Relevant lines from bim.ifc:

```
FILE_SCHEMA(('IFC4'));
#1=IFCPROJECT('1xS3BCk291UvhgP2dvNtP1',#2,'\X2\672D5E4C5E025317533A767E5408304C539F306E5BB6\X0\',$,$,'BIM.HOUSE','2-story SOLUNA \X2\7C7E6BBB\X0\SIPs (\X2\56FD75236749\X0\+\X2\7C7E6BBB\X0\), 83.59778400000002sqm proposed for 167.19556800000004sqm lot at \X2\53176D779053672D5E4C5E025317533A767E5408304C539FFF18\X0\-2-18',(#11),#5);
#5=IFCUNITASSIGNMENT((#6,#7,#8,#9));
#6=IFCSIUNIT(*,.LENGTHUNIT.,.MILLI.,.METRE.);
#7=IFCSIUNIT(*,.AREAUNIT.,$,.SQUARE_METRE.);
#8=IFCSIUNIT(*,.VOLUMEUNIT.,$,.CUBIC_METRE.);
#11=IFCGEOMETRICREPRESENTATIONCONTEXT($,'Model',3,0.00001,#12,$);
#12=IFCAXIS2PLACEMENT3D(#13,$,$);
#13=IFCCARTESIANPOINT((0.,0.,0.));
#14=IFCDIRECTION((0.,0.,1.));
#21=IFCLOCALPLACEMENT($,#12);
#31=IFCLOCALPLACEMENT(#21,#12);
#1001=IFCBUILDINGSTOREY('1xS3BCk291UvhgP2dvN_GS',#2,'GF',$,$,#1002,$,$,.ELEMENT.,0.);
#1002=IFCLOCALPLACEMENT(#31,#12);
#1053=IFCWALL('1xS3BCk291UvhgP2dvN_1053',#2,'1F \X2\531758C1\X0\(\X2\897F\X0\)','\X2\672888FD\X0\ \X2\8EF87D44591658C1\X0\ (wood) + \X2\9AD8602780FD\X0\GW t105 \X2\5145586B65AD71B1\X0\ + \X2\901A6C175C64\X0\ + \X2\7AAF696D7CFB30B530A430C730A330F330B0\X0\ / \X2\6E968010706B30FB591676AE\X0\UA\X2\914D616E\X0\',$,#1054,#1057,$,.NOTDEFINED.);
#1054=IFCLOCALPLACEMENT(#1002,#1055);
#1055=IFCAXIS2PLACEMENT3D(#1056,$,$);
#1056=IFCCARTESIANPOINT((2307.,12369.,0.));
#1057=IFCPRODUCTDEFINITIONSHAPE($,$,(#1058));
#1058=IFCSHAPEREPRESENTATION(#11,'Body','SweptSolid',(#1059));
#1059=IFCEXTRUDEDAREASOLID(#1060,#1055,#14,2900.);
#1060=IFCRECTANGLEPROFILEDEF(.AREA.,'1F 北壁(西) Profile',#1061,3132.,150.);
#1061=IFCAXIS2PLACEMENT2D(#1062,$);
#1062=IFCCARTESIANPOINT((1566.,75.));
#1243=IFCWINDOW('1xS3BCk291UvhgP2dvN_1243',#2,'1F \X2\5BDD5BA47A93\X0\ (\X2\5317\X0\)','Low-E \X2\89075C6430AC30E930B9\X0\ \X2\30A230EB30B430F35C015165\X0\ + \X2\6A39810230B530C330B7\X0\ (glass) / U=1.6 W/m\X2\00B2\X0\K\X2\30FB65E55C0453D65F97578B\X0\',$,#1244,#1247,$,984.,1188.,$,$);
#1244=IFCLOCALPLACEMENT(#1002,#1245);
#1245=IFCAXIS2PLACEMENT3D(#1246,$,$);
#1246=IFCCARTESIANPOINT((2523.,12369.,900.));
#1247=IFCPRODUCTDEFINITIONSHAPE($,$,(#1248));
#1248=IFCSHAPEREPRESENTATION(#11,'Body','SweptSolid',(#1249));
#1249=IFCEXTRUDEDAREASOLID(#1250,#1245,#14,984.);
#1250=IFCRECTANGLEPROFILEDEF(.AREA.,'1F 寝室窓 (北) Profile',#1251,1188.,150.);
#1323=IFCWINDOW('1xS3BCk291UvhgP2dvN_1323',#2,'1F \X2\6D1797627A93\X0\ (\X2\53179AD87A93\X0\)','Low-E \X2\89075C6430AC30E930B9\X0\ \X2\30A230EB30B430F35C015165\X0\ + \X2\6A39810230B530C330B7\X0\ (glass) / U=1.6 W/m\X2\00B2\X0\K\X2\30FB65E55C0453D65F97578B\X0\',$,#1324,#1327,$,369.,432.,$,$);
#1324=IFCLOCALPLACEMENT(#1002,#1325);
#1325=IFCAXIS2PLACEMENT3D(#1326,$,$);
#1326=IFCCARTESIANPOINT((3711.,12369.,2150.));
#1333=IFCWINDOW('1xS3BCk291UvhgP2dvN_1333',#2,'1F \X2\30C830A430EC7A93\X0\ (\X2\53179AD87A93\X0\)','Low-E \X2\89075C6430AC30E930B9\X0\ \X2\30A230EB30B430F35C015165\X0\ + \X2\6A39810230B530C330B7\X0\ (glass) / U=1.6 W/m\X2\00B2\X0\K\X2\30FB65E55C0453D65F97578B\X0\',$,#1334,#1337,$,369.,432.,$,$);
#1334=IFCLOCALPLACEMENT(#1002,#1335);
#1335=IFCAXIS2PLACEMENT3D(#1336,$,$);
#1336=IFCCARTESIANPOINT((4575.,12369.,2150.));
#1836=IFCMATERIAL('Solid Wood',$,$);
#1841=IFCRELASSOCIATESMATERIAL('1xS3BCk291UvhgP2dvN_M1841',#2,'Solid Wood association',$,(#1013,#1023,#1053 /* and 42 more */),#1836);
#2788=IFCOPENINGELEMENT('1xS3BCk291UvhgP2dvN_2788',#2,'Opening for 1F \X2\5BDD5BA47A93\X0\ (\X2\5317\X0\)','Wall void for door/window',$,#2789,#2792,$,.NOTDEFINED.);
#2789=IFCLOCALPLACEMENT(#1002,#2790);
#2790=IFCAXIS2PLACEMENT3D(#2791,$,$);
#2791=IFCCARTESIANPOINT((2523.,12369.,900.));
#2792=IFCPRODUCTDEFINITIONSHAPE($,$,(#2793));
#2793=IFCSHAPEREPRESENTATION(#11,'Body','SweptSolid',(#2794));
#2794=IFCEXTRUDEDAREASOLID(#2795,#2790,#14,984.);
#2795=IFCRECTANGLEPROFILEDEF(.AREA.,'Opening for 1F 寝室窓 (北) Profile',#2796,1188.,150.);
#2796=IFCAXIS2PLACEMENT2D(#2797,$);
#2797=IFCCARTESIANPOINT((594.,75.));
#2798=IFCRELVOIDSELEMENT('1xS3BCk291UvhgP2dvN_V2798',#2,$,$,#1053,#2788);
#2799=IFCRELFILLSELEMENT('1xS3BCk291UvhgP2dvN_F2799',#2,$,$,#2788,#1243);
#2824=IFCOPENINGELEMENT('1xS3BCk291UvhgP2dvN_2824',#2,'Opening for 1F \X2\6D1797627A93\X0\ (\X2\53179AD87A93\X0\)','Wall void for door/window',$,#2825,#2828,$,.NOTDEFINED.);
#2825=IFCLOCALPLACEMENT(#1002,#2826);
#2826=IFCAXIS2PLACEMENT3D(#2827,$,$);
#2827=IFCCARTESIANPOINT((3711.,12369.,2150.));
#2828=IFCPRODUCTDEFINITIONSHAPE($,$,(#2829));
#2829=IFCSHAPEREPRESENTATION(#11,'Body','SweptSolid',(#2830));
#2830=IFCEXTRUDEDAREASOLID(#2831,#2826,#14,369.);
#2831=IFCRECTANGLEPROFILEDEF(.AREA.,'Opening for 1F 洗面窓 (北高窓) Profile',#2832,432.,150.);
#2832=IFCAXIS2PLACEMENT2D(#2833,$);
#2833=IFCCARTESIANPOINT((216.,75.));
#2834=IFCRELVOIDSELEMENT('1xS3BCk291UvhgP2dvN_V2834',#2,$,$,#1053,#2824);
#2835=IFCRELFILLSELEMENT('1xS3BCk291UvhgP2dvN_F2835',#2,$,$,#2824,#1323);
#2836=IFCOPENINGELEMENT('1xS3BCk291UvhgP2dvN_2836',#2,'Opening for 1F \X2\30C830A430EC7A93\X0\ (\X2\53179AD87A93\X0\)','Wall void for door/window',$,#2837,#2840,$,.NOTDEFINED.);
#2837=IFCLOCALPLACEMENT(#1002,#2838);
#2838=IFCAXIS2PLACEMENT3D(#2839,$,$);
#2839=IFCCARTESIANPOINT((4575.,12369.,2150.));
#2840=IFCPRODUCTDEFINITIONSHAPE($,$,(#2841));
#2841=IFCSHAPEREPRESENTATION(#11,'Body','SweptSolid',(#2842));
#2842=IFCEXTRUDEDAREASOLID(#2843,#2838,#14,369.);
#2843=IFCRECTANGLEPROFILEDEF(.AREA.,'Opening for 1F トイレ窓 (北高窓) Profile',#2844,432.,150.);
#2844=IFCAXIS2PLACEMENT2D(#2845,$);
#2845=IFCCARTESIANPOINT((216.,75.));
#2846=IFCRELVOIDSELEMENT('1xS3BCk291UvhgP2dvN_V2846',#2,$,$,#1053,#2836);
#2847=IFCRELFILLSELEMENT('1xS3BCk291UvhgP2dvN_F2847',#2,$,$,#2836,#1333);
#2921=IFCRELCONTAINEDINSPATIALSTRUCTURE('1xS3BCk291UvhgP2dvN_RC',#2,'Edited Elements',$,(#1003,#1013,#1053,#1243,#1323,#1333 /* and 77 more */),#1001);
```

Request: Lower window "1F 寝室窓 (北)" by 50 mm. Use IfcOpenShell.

```python
import numpy as np
import ifcopenshell
import ifcopenshell.api.geometry
import ifcopenshell.util.placement
import ifcopenshell.util.unit

model = ifcopenshell.open("bim.ifc")
unit_scale = ifcopenshell.util.unit.calculate_unit_scale(model)

window = model.by_guid("1xS3BCk291UvhgP2dvN_1243")
opening = window.FillsVoids[0].RelatingOpeningElement
dz = -50.0

shift = np.array([0.0, 0.0, dz])
# The window is not placed relative to its opening, so move both.
for product in (opening, window):
    matrix = ifcopenshell.util.placement.get_local_placement(product.ObjectPlacement)
    matrix[:3, 3] += shift
    ifcopenshell.api.geometry.edit_object_placement(model, product=product, matrix=matrix, is_si=False)

print(f"moved by {dz * unit_scale:+.3f} m")

model.write("bim_edited.ifc")
```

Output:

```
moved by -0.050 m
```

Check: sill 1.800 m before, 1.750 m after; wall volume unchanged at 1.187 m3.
